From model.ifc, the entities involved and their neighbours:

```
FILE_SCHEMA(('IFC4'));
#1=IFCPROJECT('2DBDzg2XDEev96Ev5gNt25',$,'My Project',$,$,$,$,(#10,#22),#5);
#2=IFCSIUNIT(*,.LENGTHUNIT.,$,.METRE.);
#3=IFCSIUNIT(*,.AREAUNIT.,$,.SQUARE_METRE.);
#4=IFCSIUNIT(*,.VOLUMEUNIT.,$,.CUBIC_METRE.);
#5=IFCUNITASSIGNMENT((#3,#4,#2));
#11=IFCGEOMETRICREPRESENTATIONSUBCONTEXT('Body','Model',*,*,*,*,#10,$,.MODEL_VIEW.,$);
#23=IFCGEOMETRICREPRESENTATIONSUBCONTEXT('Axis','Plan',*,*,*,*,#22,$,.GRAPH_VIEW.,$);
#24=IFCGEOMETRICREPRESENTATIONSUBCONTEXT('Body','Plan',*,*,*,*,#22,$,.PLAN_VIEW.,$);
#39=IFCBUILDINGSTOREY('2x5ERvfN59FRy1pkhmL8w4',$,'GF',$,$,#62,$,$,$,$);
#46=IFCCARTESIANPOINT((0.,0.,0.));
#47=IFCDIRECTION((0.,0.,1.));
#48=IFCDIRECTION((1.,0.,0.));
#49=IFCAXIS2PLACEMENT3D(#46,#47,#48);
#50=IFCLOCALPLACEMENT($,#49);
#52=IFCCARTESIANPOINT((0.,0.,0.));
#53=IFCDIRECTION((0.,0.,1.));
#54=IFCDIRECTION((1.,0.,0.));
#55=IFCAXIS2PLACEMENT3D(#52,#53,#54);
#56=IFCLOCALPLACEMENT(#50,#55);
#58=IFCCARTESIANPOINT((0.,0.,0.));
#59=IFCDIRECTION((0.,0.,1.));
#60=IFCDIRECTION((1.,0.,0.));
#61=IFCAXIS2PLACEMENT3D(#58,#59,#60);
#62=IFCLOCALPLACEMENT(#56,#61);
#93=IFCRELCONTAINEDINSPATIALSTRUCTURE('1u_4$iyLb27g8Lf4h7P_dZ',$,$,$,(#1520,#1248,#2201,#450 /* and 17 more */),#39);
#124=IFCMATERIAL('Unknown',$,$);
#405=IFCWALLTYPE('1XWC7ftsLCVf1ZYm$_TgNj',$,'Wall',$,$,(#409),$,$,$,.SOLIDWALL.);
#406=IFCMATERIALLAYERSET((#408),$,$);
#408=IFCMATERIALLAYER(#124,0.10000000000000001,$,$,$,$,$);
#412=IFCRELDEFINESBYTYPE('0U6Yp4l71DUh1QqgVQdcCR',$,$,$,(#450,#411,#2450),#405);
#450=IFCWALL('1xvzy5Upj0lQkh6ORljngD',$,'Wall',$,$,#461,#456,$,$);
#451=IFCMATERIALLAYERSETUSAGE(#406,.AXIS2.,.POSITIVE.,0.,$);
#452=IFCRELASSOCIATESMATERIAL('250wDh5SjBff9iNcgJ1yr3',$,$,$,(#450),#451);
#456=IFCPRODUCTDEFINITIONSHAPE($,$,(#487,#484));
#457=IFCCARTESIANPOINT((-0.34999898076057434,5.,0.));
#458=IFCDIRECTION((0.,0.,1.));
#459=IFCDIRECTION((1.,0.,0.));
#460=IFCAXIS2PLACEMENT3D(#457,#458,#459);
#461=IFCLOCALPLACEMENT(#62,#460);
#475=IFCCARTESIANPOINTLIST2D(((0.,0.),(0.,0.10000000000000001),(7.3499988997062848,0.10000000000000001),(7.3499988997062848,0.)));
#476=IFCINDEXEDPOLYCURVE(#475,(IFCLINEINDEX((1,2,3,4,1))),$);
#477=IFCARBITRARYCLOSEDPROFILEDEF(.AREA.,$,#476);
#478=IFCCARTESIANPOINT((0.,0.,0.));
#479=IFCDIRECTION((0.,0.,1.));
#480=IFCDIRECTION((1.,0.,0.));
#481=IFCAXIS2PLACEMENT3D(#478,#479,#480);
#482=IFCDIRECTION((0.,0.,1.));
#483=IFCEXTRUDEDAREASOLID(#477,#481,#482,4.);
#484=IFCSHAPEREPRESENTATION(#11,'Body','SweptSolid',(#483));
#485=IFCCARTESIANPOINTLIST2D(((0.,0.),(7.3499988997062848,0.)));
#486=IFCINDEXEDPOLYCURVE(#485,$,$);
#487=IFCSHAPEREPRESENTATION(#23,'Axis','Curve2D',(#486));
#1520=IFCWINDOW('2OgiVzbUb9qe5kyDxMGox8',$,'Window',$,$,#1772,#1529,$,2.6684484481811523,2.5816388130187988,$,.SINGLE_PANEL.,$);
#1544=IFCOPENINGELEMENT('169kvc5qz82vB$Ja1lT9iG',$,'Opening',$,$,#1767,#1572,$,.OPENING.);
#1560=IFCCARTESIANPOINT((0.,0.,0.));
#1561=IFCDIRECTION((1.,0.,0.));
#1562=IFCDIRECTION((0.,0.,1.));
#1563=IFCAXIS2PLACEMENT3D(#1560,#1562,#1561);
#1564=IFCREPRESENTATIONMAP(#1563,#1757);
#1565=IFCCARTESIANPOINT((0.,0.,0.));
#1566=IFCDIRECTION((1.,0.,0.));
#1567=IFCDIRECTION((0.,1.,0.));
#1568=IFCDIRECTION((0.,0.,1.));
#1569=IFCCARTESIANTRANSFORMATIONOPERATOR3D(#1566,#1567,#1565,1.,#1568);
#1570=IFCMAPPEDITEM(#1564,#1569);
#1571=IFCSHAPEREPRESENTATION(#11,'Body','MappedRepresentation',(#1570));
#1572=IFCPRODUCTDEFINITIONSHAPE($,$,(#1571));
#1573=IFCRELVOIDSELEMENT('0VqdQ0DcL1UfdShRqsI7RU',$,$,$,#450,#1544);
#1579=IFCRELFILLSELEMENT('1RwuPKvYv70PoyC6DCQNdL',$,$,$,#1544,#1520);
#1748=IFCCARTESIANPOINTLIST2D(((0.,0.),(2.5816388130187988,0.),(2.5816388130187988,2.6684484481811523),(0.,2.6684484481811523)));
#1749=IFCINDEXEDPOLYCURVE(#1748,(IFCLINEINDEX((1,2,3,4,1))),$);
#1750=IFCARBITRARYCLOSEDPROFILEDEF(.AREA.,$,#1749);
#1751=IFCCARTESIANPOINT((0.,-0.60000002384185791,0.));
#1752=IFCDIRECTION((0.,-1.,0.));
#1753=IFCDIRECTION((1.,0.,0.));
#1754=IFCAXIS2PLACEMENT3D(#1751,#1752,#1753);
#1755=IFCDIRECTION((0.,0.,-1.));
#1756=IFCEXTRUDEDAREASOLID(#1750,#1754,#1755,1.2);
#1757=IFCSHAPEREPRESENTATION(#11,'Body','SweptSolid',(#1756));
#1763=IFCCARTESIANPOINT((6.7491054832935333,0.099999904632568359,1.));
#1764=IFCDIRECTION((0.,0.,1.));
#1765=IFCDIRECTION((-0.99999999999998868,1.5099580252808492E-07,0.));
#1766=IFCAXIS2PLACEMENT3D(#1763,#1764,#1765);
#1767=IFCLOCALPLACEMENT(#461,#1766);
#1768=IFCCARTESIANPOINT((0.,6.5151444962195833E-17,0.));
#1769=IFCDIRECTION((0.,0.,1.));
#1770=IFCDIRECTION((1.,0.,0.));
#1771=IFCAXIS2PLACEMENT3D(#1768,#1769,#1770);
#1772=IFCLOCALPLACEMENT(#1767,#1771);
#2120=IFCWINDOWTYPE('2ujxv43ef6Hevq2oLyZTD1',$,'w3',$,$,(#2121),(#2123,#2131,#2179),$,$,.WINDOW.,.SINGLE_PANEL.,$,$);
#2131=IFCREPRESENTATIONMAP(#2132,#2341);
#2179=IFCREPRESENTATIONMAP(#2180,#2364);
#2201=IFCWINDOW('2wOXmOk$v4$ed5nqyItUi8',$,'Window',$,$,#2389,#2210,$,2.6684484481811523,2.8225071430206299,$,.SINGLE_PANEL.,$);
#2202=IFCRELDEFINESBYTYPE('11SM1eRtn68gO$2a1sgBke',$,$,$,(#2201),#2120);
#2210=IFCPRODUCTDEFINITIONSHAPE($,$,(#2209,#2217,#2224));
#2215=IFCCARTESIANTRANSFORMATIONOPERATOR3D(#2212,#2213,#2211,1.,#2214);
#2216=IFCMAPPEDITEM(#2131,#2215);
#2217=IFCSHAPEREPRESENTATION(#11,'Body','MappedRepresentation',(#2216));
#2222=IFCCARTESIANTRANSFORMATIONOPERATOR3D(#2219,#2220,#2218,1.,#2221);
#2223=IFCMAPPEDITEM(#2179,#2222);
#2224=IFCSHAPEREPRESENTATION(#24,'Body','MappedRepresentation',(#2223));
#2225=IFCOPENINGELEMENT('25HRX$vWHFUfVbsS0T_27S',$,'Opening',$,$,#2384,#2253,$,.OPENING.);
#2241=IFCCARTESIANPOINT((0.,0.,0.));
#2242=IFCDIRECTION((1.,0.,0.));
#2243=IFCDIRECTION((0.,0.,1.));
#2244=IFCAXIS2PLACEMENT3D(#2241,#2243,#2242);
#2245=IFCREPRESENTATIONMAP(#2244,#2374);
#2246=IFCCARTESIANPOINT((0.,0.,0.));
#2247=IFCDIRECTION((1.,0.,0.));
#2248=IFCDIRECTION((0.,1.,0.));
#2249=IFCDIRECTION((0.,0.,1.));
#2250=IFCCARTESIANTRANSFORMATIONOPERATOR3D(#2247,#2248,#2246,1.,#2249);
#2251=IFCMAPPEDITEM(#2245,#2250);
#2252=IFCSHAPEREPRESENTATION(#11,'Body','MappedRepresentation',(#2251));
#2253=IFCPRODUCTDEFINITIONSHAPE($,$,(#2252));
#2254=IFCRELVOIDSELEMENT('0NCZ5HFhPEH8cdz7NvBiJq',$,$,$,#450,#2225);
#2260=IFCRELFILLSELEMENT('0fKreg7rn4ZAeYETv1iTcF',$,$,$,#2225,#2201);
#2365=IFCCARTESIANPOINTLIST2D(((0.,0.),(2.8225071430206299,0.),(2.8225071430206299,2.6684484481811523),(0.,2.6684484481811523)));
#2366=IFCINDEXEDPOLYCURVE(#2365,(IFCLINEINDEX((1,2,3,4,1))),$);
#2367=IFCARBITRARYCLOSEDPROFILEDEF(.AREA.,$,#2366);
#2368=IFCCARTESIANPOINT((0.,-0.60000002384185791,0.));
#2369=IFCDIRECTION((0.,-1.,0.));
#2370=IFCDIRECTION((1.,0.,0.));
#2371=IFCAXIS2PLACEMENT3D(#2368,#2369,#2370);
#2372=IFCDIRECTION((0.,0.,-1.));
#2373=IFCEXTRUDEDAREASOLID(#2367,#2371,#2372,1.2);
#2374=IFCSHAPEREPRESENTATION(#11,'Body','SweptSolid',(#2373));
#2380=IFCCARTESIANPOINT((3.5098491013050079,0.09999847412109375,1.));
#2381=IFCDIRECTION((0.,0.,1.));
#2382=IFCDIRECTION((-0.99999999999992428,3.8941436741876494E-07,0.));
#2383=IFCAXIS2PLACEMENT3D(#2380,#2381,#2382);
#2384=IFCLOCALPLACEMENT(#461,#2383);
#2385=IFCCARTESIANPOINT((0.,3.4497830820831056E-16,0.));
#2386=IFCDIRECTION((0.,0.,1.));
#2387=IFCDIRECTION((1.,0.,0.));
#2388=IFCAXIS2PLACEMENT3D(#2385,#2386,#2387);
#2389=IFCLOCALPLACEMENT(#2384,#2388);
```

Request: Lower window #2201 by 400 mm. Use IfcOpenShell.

```python
import numpy as np
import ifcopenshell
import ifcopenshell.api.geometry
import ifcopenshell.util.placement
import ifcopenshell.util.unit

model = ifcopenshell.open("model.ifc")
unit_scale = ifcopenshell.util.unit.calculate_unit_scale(model)

window = model.by_guid("2wOXmOk$v4$ed5nqyItUi8")
opening = window.FillsVoids[0].RelatingOpeningElement
dz = -0.4

shift = np.array([0.0, 0.0, dz])
# The window is placed relative to its opening, so it follows when the opening moves.
matrix = ifcopenshell.util.placement.get_local_placement(opening.ObjectPlacement)
matrix[:3, 3] += shift
ifcopenshell.api.geometry.edit_object_placement(
    model, product=opening, matrix=matrix, is_si=False, should_transform_children=True
)

print(f"moved by {dz * unit_scale:+.3f} m")

model.write("model_rev.ifc")
```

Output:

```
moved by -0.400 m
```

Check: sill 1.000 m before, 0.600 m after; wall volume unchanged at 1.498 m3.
